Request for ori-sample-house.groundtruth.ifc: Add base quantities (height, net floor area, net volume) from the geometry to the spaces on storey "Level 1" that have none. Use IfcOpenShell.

First a look at what the model holds.

```python
import ifcopenshell
import ifcopenshell.util.element
import ifcopenshell.util.unit

model = ifcopenshell.open("ori-sample-house.groundtruth.ifc")
print(model.schema)
for unit_type in ("LENGTHUNIT", "AREAUNIT", "VOLUMEUNIT"):
    print(unit_type, ifcopenshell.util.unit.calculate_unit_scale(model, unit_type))
storey = next(s for s in model.by_type("IfcBuildingStorey") if s.Name == "Level 1")
spaces = [e for e in ifcopenshell.util.element.get_decomposition(storey) if e.is_a("IfcSpace")]
for e in sorted(spaces, key=lambda e: e.id()):
    print(e.id(), e.is_a(), e.Name, list(ifcopenshell.util.element.get_psets(e, qtos_only=True)), sep=" | ")
```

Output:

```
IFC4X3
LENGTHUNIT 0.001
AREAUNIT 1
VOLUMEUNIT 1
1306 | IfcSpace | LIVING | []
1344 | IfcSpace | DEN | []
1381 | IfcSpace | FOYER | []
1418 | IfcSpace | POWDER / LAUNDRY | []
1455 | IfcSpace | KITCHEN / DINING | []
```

```python
import ifcopenshell
import ifcopenshell.api.pset
import ifcopenshell.geom
import ifcopenshell.util.element
import ifcopenshell.util.shape
import ifcopenshell.util.unit

model = ifcopenshell.open("ori-sample-house.groundtruth.ifc")
unit_scale = ifcopenshell.util.unit.calculate_unit_scale(model)
area_scale = ifcopenshell.util.unit.calculate_unit_scale(model, "AREAUNIT")
volume_scale = ifcopenshell.util.unit.calculate_unit_scale(model, "VOLUMEUNIT")
settings = ifcopenshell.geom.settings()

storey = next(s for s in model.by_type("IfcBuildingStorey") if s.Name == "Level 1")
spaces = [e for e in ifcopenshell.util.element.get_decomposition(storey) if e.is_a("IfcSpace")]

for e in sorted(spaces, key=lambda e: e.id()):
    if ifcopenshell.util.element.get_psets(e, qtos_only=True, should_inherit=False):
        continue
    # Geometry comes back in metres, in the element's own axes.
    shape = ifcopenshell.geom.create_shape(settings, e)
    values = {
        "Height": ifcopenshell.util.shape.get_z(shape.geometry) / unit_scale,
        "NetFloorArea": ifcopenshell.util.shape.get_footprint_area(shape.geometry) / area_scale,
        "NetVolume": ifcopenshell.util.shape.get_volume(shape.geometry) / volume_scale,
    }
    qto = ifcopenshell.api.pset.add_qto(model, product=e, name="Qto_SpaceBaseQuantities")
    ifcopenshell.api.pset.edit_qto(model, qto=qto, properties=values)
    print(e.id(), {k: round(v, 3) for k, v in values.items()})

model.write("ori-sample-house.groundtruth_rev.ifc")
```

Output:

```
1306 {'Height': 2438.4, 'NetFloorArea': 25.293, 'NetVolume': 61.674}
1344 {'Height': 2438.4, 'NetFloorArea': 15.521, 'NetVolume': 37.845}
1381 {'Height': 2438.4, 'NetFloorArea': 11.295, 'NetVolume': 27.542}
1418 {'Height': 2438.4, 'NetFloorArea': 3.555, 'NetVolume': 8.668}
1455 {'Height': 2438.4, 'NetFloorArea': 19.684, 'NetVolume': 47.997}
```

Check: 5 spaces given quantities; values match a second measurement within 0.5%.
